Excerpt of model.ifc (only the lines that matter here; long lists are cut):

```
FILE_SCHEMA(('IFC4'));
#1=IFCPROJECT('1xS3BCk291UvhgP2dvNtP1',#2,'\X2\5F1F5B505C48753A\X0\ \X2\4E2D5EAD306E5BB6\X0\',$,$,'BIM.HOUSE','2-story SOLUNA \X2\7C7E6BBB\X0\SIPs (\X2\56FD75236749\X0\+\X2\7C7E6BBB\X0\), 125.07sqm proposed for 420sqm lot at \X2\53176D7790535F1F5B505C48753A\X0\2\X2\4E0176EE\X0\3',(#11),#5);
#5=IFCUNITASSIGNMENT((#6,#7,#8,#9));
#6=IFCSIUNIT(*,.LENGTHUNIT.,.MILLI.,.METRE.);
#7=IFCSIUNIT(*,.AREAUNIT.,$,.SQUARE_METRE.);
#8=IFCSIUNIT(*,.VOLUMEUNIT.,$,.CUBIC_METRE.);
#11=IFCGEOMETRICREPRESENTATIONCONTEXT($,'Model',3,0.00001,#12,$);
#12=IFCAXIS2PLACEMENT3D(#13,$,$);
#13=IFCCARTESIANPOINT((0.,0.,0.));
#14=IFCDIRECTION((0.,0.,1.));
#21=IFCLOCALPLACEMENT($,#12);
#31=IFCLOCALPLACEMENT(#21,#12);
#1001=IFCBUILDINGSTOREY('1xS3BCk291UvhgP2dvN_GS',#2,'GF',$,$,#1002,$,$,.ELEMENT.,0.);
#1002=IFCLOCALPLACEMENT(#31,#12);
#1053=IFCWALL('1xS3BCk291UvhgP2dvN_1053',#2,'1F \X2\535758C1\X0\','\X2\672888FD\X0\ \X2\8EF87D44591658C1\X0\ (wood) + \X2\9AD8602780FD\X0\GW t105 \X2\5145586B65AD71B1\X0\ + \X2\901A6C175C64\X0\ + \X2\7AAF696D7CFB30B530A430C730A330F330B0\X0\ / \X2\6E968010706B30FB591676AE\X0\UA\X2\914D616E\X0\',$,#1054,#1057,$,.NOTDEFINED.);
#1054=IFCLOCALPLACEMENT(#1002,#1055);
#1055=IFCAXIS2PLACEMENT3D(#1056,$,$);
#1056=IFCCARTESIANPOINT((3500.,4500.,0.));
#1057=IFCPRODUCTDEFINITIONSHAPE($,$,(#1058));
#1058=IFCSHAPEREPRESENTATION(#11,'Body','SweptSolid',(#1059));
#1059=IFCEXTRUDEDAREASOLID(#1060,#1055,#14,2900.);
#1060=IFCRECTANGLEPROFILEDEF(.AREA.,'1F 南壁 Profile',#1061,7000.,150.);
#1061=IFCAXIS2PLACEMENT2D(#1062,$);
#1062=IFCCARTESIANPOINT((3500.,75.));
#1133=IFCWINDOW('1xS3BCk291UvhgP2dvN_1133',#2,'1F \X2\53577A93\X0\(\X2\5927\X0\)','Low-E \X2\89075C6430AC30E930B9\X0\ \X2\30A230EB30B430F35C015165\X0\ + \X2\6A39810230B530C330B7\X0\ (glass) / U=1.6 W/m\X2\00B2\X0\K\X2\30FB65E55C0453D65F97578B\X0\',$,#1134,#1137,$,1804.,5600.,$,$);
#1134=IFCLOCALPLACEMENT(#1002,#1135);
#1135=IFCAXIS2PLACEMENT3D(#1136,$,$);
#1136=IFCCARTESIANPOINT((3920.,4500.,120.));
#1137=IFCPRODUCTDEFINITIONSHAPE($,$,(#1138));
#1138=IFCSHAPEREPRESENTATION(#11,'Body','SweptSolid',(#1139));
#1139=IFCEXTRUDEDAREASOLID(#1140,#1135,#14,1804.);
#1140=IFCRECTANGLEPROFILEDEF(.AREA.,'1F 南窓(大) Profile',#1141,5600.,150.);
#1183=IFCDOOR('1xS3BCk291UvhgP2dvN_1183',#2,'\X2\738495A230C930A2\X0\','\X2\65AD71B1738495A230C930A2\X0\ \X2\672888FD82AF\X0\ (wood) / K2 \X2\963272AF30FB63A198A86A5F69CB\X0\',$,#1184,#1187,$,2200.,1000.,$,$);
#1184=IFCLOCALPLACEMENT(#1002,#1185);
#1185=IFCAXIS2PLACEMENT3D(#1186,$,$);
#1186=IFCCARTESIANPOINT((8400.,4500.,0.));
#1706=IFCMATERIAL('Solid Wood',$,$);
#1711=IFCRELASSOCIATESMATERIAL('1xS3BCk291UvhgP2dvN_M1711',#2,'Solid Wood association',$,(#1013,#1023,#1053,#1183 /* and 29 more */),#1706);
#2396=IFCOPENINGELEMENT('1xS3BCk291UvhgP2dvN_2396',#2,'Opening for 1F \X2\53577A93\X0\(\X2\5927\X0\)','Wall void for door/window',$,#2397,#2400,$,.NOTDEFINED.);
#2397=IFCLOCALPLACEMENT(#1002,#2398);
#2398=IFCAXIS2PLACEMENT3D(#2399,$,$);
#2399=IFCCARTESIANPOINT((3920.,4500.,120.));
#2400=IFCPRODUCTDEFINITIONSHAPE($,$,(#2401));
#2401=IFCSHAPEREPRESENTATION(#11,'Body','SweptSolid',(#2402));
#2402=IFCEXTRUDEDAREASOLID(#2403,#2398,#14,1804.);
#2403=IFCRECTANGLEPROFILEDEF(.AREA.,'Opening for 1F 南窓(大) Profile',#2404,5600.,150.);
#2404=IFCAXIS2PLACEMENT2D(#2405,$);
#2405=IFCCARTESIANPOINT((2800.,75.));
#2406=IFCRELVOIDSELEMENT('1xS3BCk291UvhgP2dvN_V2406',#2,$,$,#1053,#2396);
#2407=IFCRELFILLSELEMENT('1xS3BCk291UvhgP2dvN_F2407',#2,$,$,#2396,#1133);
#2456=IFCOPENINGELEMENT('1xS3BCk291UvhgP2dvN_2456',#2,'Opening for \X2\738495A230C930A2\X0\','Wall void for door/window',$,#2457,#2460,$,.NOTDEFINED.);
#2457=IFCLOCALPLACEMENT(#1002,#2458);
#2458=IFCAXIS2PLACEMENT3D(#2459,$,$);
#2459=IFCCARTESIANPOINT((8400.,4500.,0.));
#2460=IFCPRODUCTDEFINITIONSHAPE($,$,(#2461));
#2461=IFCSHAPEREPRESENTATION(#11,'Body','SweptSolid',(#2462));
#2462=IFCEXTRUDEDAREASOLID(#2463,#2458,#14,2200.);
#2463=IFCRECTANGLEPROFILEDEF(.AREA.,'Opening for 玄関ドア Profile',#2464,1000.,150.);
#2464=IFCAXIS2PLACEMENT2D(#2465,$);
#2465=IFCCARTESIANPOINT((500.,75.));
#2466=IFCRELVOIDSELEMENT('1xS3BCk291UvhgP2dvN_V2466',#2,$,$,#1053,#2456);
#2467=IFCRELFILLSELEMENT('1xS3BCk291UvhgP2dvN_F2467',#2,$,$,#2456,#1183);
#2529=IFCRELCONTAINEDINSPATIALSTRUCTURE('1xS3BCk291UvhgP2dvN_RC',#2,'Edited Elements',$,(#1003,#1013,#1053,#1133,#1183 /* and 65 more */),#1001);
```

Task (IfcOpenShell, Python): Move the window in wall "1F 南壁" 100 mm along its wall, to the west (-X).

```python
import ifcopenshell
import ifcopenshell.api.geometry
import ifcopenshell.util.placement
import ifcopenshell.util.unit

model = ifcopenshell.open("model.ifc")
unit_scale = ifcopenshell.util.unit.calculate_unit_scale(model)

window = model.by_guid("1xS3BCk291UvhgP2dvN_1133")
opening = window.FillsVoids[0].RelatingOpeningElement
wall = opening.VoidsElements[0].RelatingBuildingElement

wall_matrix = ifcopenshell.util.placement.get_local_placement(wall.ObjectPlacement)
shift = wall_matrix[:3, 0] * -0.1 / unit_scale
before = ifcopenshell.util.placement.get_local_placement(window.ObjectPlacement)[:3, 3].copy()

# The window is not placed relative to its opening, so move both.
for product in (opening, window):
    matrix = ifcopenshell.util.placement.get_local_placement(product.ObjectPlacement)
    matrix[:3, 3] += shift
    ifcopenshell.api.geometry.edit_object_placement(model, product=product, matrix=matrix, is_si=False)

after = ifcopenshell.util.placement.get_local_placement(window.ObjectPlacement)[:3, 3]
print("window moved by", (after - before).round(3) + 0.0)

model.write("model_v2.ifc")
```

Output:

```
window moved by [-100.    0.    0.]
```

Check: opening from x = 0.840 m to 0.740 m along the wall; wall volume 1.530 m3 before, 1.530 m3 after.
